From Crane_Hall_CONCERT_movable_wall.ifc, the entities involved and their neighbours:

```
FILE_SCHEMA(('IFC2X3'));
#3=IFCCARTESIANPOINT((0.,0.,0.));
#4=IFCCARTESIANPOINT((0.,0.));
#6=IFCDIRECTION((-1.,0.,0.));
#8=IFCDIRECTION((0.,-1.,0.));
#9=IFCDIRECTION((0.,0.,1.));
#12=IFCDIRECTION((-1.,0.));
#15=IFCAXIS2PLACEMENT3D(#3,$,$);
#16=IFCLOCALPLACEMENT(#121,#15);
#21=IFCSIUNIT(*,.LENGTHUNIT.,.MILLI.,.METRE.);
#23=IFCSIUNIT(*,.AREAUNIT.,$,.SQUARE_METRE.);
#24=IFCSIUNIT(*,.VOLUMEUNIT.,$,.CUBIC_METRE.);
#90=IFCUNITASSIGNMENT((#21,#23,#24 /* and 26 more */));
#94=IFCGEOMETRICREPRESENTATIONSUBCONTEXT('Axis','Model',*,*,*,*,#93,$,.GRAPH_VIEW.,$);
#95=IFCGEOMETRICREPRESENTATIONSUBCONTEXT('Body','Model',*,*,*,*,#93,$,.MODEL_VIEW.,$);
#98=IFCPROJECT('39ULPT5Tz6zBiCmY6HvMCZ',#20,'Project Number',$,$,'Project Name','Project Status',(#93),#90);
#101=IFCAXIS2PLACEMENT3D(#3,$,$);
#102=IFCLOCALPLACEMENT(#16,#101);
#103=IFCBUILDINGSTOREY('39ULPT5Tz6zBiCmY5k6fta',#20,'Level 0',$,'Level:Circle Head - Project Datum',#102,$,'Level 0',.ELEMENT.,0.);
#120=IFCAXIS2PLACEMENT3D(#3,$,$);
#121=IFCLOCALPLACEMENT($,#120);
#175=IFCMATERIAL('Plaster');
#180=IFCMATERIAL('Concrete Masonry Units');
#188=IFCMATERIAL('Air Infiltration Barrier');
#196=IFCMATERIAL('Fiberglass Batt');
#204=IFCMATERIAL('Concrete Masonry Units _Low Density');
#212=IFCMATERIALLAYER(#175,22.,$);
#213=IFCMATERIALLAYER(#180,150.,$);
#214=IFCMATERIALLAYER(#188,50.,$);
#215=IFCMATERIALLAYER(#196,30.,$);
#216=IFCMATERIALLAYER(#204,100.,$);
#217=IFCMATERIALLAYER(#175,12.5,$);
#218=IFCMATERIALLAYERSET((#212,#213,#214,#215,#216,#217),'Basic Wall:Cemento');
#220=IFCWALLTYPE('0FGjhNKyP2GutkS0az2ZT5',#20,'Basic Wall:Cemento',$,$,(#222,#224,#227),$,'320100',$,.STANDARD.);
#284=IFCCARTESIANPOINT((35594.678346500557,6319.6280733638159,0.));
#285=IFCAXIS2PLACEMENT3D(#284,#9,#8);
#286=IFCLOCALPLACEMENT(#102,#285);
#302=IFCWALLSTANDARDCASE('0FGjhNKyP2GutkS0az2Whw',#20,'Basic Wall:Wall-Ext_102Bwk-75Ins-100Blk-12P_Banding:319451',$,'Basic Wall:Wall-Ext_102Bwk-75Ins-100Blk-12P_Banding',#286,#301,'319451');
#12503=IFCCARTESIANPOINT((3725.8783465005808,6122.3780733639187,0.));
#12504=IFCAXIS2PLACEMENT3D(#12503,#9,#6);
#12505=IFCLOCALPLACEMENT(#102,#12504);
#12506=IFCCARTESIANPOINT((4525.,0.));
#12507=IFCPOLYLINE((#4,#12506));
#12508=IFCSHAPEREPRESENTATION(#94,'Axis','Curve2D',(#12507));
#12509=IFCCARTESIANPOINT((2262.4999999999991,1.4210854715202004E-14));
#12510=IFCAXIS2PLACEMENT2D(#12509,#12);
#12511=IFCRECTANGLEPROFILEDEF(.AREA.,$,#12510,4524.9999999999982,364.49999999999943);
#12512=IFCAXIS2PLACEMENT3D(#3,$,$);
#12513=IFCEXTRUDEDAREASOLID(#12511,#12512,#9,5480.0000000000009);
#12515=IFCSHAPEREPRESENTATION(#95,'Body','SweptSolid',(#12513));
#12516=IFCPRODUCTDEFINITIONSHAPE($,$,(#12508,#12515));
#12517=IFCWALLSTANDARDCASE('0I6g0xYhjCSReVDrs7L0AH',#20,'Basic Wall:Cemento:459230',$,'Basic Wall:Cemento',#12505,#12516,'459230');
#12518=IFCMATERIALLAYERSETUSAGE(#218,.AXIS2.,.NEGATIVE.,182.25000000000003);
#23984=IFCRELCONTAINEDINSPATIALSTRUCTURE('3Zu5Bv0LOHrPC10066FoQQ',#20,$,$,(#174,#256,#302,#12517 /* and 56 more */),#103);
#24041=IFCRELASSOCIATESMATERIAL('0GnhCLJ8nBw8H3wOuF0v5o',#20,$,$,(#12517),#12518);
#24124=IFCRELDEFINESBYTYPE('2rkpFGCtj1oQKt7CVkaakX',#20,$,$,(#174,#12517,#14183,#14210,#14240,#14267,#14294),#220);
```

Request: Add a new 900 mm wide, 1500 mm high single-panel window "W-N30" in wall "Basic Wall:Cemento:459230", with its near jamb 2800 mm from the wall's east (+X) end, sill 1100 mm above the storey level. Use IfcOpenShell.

```python
import numpy as np
import ifcopenshell
import ifcopenshell.api.feature
import ifcopenshell.api.geometry
import ifcopenshell.api.root
import ifcopenshell.api.spatial
import ifcopenshell.api.type
import ifcopenshell.geom
import ifcopenshell.util.element
import ifcopenshell.util.placement
import ifcopenshell.util.representation
import ifcopenshell.util.shape
import ifcopenshell.util.unit

model = ifcopenshell.open("Crane_Hall_CONCERT_movable_wall.ifc")
unit_scale = ifcopenshell.util.unit.calculate_unit_scale(model)
settings = ifcopenshell.geom.settings()


def volume(element):
    """Net volume in cubic metres, openings subtracted."""
    shape = ifcopenshell.geom.create_shape(settings, element)
    return ifcopenshell.util.shape.get_volume(shape.geometry)


wall = model.by_guid("0I6g0xYhjCSReVDrs7L0AH")
storey = ifcopenshell.util.element.get_container(wall, ifc_class="IfcBuildingStorey")
context = ifcopenshell.util.representation.get_context(model, "Model", "Body", "MODEL_VIEW")
before = volume(wall)

width, height, from_end, sill = 0.9, 1.5, 2.8, 1.1  # metres

# The wall runs along its own X axis, and the end named is its -X end.
wall_shape = ifcopenshell.geom.create_shape(settings, wall)
x, y, z = ifcopenshell.util.shape.get_vertices(wall_shape.geometry).T
start = x.min() + from_end
face, thickness = float(y.min()), float(y.max() - y.min())
wall_matrix = ifcopenshell.util.placement.get_local_placement(wall.ObjectPlacement)
level = ifcopenshell.util.placement.get_local_placement(storey.ObjectPlacement)[2, 3]


def in_wall(x, y):
    """Placement at x, y metres in the wall's axes, at sill height."""
    matrix = wall_matrix.copy()
    matrix[:, 3] = wall_matrix @ np.array([x / unit_scale, y / unit_scale, 0.0, 1.0])
    matrix[2, 3] = level + sill / unit_scale
    return matrix


# Opening: a box that overshoots both wall faces by 50 mm.
opening = ifcopenshell.api.root.create_entity(model, ifc_class="IfcOpeningElement")
box = ifcopenshell.api.geometry.add_wall_representation(
    model, context=context, length=width, height=height, thickness=thickness + 0.1
)
ifcopenshell.api.geometry.assign_representation(model, product=opening, representation=box)
ifcopenshell.api.geometry.edit_object_placement(model, product=opening, matrix=in_wall(start, face - 0.05), is_si=False)
ifcopenshell.api.feature.add_feature(model, feature=opening, element=wall)

window = ifcopenshell.api.root.create_entity(model, ifc_class="IfcWindow", name="W-N30")
window.OverallWidth, window.OverallHeight = width / unit_scale, height / unit_scale
body = ifcopenshell.api.geometry.add_window_representation(
    model,
    context=context,
    overall_width=window.OverallWidth,
    overall_height=window.OverallHeight,
    partition_type="SINGLE_PANEL",
)
ifcopenshell.api.geometry.assign_representation(model, product=window, representation=body)
ifcopenshell.api.spatial.assign_container(model, products=[window], relating_structure=storey)
fills = ifcopenshell.api.feature.add_filling(model, opening=opening, element=window)
fills.OwnerHistory = window.OwnerHistory  # required in IFC2X3

# IFC2X3 keeps the operation on the window style.
style = ifcopenshell.api.root.create_entity(model, ifc_class="IfcWindowStyle", name="W-N30")
style.OperationType, style.ConstructionType = "SINGLE_PANEL", "NOTDEFINED"
style.ParameterTakesPrecedence = style.Sizeable = False
ifcopenshell.api.type.assign_type(model, related_objects=[window], relating_type=style)

# Centre the window in the wall's thickness.
ifcopenshell.api.geometry.edit_object_placement(model, product=window, matrix=in_wall(start, face), is_si=False)
window_shape = ifcopenshell.geom.create_shape(settings, window)
depth = ifcopenshell.util.shape.get_vertices(window_shape.geometry)[:, 1]
offset = face + thickness / 2 - (depth.min() + depth.max()) / 2
ifcopenshell.api.geometry.edit_object_placement(model, product=window, matrix=in_wall(start, offset), is_si=False)

after = volume(wall)

print(f"wall volume {before:.3f} -> {after:.3f} m3")

model.write("Crane_Hall_CONCERT_movable_wall_rev.ifc")
```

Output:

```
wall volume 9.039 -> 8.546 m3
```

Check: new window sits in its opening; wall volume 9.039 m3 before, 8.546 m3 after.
